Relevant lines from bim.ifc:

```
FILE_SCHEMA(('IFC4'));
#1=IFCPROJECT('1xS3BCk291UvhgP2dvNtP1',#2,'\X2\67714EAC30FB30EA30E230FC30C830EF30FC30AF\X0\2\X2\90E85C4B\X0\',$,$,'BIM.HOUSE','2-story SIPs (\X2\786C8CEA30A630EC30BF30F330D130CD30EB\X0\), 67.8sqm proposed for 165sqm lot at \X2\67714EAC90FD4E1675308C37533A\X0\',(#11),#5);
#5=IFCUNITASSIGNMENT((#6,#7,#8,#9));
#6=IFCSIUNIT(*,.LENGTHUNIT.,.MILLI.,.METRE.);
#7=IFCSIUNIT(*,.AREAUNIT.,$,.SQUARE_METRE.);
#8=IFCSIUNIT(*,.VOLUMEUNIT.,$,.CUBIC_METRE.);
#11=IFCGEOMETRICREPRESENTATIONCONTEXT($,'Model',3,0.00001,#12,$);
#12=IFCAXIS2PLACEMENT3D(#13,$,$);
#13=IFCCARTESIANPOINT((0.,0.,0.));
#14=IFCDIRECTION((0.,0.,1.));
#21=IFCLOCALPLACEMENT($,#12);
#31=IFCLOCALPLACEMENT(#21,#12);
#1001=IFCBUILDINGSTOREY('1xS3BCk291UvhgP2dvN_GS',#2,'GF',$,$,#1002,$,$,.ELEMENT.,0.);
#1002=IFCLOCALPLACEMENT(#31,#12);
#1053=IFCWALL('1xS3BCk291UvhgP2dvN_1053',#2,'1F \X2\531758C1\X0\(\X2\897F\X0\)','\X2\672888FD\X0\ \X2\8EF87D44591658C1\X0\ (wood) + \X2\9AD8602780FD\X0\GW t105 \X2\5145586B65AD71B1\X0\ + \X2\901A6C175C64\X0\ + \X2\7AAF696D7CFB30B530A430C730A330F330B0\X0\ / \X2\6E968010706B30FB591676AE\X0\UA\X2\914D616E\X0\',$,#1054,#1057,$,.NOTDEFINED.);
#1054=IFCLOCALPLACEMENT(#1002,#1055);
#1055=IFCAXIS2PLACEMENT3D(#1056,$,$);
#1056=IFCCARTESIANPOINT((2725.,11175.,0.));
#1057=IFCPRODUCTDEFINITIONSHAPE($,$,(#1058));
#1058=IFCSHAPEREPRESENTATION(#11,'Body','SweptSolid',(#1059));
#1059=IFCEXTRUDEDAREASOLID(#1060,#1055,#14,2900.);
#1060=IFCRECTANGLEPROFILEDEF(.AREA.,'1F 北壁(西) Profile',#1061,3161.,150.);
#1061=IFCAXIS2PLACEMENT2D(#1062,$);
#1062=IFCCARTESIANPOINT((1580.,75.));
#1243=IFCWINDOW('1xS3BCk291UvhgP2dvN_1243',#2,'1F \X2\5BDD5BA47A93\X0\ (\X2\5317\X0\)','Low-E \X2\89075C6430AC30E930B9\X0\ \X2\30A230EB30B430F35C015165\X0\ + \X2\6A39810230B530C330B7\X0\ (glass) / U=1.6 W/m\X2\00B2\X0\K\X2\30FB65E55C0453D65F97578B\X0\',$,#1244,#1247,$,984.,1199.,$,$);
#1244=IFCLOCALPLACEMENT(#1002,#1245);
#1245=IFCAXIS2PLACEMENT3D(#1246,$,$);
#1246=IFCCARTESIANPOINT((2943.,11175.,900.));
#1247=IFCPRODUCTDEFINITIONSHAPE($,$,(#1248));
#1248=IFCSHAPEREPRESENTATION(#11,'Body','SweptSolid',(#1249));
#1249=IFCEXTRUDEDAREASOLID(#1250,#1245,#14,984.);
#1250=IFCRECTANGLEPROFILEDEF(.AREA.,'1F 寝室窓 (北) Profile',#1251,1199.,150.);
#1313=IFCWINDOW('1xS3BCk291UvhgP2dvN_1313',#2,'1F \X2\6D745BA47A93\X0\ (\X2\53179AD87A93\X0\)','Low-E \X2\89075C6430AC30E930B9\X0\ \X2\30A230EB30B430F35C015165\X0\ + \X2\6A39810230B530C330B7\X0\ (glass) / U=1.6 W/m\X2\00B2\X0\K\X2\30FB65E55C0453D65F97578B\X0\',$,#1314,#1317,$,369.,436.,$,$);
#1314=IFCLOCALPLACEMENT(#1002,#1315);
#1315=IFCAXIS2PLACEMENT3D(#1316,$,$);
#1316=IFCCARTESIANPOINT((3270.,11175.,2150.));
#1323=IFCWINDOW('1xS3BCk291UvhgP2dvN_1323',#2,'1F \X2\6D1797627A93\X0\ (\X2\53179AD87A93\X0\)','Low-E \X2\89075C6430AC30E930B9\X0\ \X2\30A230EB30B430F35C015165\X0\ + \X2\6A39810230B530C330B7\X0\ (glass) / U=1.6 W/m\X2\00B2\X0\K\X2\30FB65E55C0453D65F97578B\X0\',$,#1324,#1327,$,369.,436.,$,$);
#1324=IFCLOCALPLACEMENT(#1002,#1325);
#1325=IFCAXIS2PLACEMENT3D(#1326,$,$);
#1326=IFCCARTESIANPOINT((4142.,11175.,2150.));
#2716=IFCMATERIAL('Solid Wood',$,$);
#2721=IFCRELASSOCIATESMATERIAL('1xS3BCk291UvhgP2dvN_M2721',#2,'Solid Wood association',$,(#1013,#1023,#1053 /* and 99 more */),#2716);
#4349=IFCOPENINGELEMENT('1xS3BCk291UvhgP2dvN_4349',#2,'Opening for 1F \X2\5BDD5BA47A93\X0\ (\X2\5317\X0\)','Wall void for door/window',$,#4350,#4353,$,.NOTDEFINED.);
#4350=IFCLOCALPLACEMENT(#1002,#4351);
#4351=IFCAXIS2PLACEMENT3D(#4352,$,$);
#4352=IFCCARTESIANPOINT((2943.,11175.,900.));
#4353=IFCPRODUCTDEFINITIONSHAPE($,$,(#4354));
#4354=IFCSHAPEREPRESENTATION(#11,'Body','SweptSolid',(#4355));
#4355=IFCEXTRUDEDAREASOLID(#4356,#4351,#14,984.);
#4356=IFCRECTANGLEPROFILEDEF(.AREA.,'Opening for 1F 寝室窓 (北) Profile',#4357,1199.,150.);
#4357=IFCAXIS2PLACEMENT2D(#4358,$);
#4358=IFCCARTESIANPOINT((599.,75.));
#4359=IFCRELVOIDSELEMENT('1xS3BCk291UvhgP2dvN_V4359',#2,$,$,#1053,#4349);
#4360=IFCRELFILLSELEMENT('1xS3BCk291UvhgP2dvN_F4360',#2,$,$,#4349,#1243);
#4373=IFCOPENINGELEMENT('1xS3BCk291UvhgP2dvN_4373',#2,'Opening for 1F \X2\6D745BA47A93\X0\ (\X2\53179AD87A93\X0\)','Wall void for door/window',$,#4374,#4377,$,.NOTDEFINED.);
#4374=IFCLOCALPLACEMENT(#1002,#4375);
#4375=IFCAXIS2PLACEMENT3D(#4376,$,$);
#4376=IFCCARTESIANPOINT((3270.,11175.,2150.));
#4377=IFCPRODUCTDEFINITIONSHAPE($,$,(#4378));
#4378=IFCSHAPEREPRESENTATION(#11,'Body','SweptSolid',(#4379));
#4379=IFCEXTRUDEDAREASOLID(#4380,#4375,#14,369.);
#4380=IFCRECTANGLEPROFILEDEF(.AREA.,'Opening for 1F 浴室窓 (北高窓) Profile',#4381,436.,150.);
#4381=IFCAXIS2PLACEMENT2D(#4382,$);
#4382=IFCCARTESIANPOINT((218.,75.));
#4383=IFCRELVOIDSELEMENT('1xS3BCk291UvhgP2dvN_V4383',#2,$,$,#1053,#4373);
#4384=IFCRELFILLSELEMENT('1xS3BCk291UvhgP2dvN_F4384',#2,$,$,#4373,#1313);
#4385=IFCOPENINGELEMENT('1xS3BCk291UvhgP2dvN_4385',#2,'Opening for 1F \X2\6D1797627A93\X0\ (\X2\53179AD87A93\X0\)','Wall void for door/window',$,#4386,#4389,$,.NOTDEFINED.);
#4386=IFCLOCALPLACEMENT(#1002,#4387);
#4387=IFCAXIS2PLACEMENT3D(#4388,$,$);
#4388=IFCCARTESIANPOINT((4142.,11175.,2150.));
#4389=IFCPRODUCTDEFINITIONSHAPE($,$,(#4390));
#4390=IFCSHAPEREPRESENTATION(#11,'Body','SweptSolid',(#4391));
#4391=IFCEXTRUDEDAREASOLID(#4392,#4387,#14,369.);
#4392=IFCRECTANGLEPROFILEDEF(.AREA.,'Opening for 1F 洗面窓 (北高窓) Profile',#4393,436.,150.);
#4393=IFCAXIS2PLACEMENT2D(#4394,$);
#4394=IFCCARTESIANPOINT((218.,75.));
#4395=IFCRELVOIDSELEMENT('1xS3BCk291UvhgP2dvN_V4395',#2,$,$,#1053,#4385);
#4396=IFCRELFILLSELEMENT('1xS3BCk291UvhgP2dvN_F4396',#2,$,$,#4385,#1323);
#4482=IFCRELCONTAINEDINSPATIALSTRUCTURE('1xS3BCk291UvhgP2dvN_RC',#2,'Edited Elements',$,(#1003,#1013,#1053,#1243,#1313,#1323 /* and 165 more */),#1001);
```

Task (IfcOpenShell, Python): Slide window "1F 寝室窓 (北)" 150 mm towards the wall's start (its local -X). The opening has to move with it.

```python
import ifcopenshell
import ifcopenshell.api.geometry
import ifcopenshell.util.placement

model = ifcopenshell.open("bim.ifc")

window = model.by_id(1243)
opening = window.FillsVoids[0].RelatingOpeningElement
wall = opening.VoidsElements[0].RelatingBuildingElement

wall_matrix = ifcopenshell.util.placement.get_local_placement(wall.ObjectPlacement)
shift = wall_matrix[:3, 0] * -150.0
before = ifcopenshell.util.placement.get_local_placement(window.ObjectPlacement)[:3, 3].copy()

# The window is not placed relative to its opening, so move both.
for product in (opening, window):
    matrix = ifcopenshell.util.placement.get_local_placement(product.ObjectPlacement)
    matrix[:3, 3] += shift
    ifcopenshell.api.geometry.edit_object_placement(model, product=product, matrix=matrix, is_si=False)

after = ifcopenshell.util.placement.get_local_placement(window.ObjectPlacement)[:3, 3]
print("window moved by", (after - before).round(3) + 0.0)

model.write("bim-out.ifc")
```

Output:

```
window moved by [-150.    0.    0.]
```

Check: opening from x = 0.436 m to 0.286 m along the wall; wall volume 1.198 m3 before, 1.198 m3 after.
